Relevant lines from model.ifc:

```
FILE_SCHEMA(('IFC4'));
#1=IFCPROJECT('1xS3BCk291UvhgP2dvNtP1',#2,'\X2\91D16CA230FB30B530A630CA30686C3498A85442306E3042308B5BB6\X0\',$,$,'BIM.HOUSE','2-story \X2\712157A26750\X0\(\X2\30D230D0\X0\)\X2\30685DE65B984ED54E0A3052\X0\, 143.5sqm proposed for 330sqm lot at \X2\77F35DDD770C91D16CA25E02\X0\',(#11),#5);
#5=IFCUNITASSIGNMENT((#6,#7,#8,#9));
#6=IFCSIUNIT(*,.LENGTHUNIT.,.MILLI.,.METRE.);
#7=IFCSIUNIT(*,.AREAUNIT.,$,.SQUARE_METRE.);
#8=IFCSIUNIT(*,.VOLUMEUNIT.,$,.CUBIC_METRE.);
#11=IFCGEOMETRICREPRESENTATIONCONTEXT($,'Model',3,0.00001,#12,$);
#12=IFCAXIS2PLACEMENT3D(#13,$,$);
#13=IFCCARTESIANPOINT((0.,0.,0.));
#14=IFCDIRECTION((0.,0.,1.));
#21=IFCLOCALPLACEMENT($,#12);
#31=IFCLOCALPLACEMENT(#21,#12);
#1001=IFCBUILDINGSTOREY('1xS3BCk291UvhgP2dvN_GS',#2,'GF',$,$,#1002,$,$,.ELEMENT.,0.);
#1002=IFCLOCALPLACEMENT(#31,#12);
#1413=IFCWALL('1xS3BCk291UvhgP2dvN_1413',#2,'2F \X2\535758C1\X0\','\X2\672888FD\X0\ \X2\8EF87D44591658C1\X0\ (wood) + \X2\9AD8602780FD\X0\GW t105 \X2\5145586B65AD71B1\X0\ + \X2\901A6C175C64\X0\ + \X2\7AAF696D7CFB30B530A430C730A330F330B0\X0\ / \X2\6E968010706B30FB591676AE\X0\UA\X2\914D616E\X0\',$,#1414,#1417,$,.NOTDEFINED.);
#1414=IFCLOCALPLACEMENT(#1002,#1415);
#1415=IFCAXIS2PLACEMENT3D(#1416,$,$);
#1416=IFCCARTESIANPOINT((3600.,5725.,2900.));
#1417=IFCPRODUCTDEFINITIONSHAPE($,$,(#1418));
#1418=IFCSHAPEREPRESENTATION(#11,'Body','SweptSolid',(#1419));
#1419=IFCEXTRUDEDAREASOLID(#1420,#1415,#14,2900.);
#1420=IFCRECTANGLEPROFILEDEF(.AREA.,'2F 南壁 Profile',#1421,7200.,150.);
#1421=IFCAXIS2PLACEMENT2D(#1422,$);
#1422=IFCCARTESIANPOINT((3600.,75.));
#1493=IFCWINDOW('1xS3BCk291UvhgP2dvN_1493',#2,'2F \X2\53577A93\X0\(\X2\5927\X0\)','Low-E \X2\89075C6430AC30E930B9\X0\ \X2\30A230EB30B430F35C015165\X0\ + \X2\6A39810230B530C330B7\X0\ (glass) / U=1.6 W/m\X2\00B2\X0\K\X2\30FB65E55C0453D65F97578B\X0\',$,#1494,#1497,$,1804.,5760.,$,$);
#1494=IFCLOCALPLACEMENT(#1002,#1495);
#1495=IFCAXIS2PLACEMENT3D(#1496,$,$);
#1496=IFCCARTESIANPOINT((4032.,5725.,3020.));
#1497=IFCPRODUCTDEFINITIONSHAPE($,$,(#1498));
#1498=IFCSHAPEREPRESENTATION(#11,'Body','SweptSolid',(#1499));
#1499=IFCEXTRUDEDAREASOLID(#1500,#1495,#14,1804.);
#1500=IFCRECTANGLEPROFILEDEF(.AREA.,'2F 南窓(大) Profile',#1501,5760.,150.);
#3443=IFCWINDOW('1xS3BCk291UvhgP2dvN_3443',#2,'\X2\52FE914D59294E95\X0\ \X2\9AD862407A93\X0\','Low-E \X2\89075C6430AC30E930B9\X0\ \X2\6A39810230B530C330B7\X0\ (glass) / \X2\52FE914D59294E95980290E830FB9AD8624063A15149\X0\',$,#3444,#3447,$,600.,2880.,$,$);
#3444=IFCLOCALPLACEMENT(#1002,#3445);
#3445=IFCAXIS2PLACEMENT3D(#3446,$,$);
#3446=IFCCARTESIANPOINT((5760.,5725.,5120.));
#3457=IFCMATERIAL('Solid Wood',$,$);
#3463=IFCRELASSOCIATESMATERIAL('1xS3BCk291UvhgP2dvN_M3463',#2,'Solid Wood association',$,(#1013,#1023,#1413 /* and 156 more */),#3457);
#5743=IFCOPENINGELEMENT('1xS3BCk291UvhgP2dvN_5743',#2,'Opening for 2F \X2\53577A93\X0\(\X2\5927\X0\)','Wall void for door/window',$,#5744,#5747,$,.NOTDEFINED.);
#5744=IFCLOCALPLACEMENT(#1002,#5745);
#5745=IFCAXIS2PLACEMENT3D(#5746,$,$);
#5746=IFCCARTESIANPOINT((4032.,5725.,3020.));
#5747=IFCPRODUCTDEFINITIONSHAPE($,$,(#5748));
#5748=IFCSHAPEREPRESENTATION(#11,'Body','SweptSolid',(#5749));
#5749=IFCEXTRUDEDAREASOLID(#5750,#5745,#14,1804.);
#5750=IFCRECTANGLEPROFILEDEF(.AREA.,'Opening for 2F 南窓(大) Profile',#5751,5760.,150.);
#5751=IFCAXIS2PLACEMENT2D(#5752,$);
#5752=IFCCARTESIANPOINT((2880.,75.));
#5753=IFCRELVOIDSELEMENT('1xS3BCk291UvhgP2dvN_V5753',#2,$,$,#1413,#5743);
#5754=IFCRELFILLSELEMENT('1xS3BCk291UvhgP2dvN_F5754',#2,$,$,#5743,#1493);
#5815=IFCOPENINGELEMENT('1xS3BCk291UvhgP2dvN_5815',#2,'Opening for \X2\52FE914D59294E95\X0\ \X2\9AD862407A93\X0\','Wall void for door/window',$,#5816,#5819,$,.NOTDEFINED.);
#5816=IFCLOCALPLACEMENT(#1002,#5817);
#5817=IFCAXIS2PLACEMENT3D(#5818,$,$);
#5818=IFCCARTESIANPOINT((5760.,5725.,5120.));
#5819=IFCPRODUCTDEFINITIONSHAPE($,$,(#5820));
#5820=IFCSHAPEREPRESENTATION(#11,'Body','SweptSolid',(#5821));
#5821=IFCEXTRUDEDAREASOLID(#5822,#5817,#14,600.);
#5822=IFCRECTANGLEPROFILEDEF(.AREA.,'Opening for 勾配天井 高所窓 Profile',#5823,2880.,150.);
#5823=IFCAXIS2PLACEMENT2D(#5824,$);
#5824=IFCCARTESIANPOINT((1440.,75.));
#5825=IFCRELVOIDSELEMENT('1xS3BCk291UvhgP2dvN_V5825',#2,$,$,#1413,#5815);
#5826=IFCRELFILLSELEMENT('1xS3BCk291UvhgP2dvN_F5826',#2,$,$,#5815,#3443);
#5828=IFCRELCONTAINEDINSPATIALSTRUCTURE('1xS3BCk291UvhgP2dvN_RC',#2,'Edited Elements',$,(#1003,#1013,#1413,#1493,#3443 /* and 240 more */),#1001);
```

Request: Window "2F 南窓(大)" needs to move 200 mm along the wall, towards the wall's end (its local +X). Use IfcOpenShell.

```python
import ifcopenshell
import ifcopenshell.api.geometry
import ifcopenshell.util.placement

model = ifcopenshell.open("model.ifc")

window = model.by_guid("1xS3BCk291UvhgP2dvN_1493")
opening = window.FillsVoids[0].RelatingOpeningElement
wall = opening.VoidsElements[0].RelatingBuildingElement

wall_matrix = ifcopenshell.util.placement.get_local_placement(wall.ObjectPlacement)
shift = wall_matrix[:3, 0] * 200.0
before = ifcopenshell.util.placement.get_local_placement(window.ObjectPlacement)[:3, 3].copy()

# The window is not placed relative to its opening, so move both.
for product in (opening, window):
    matrix = ifcopenshell.util.placement.get_local_placement(product.ObjectPlacement)
    matrix[:3, 3] += shift
    ifcopenshell.api.geometry.edit_object_placement(model, product=product, matrix=matrix, is_si=False)

after = ifcopenshell.util.placement.get_local_placement(window.ObjectPlacement)[:3, 3]
print("window moved by", (after - before).round(3) + 0.0)

model.write("model_v2.ifc")
```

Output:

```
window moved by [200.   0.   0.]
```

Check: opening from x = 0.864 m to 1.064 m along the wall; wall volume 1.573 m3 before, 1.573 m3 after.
